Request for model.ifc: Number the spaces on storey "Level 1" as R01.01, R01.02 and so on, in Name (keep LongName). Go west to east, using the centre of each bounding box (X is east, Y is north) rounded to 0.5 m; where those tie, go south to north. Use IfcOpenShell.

First a look at what the model holds.

```python
import ifcopenshell
import ifcopenshell.util.element
import ifcopenshell.util.placement

model = ifcopenshell.open("model.ifc")
print(model.schema)
storey = next(s for s in model.by_type("IfcBuildingStorey") if s.Name == "Level 1")
spaces = [e for e in ifcopenshell.util.element.get_decomposition(storey) if e.is_a("IfcSpace")]
for e in sorted(spaces, key=lambda e: e.id()):
    origin = ifcopenshell.util.placement.get_local_placement(e.ObjectPlacement)[:3, 3]
    print(e.id(), e.Name, e.LongName, origin.round(2) + 0.0, sep=" | ")
```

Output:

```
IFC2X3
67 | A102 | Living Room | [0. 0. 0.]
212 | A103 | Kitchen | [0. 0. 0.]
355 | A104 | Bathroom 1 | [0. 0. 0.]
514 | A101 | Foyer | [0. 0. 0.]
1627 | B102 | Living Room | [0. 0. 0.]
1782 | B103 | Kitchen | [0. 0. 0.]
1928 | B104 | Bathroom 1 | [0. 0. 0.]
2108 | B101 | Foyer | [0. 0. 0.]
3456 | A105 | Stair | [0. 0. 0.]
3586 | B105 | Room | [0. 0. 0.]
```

```python
import ifcopenshell
import ifcopenshell.geom
import ifcopenshell.util.element
import ifcopenshell.util.shape

model = ifcopenshell.open("model.ifc")
settings = ifcopenshell.geom.settings()
settings.set("use-world-coords", True)


def centre(element):
    shape = ifcopenshell.geom.create_shape(settings, element)
    return ifcopenshell.util.shape.get_bbox_centroid(shape.geometry)


storey = next(s for s in model.by_type("IfcBuildingStorey") if s.Name == "Level 1")
spaces = [e for e in ifcopenshell.util.element.get_decomposition(storey) if e.is_a("IfcSpace")]

# Insertion points can sit at a corner or the storey origin, so sort by the geometry (in metres).
centres = {e: centre(e) for e in spaces}
spaces.sort(key=lambda e: (round(centres[e][0] / 0.5), centres[e][1]))

for i, e in enumerate(spaces, start=1):
    number = f"R01.{i:02d}"
    e.Name = number
    print(e.id(), number)

model.write("model-out.ifc")
```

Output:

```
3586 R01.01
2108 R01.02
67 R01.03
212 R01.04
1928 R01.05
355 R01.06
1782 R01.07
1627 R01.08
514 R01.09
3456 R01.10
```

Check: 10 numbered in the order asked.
